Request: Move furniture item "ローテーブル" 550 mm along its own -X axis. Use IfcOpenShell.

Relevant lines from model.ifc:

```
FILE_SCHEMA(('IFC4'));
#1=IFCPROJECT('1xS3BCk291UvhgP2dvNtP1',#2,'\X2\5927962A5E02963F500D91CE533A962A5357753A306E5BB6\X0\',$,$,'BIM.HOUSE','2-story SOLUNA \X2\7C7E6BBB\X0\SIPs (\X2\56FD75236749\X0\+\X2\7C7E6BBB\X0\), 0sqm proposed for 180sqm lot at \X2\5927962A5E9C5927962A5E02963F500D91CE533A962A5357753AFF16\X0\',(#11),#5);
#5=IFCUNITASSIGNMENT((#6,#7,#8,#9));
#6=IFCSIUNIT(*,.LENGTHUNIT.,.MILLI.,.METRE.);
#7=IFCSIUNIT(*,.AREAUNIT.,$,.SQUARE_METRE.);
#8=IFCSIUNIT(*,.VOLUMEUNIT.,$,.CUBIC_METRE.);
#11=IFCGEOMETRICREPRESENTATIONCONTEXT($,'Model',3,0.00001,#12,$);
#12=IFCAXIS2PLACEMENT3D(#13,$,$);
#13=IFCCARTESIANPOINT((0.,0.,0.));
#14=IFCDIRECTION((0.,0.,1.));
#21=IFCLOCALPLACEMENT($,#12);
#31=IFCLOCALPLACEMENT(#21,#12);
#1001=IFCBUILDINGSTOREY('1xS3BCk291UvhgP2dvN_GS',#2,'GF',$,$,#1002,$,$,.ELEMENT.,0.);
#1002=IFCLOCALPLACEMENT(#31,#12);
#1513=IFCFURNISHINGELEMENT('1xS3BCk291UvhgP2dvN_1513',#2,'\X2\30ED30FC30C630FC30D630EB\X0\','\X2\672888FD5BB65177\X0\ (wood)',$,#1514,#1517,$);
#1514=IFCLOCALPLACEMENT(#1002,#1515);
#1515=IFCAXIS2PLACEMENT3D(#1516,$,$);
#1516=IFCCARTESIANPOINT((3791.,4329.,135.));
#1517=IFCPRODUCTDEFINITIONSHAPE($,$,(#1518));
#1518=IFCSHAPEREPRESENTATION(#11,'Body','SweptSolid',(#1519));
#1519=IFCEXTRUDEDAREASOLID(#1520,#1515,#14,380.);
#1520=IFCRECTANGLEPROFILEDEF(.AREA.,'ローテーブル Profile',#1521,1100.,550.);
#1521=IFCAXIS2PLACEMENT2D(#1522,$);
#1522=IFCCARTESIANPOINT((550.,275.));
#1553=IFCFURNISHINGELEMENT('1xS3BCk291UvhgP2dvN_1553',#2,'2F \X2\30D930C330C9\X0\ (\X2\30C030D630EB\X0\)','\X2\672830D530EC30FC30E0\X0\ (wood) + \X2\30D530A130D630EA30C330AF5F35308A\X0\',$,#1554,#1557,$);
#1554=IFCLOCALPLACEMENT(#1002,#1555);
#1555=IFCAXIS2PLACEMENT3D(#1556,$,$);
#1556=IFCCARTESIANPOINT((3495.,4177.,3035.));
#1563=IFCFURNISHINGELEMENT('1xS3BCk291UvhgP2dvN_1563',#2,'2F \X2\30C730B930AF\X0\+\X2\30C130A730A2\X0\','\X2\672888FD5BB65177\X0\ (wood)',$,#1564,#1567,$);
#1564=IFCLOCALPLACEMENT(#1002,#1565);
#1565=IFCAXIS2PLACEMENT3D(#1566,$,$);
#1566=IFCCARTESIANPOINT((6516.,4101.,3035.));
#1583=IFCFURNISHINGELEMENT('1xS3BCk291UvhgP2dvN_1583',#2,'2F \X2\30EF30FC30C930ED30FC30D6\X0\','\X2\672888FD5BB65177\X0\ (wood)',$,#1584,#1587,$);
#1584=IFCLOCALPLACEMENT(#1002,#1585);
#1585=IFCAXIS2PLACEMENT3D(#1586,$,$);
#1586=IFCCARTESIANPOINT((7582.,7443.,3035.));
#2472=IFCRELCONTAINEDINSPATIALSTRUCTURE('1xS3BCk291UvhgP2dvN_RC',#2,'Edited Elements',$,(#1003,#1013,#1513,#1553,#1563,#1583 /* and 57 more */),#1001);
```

```python
import ifcopenshell
import ifcopenshell.api.geometry
import ifcopenshell.util.placement
import ifcopenshell.util.unit

model = ifcopenshell.open("model.ifc")
unit_scale = ifcopenshell.util.unit.calculate_unit_scale(model)

item = model.by_guid("1xS3BCk291UvhgP2dvN_1513")
matrix = ifcopenshell.util.placement.get_local_placement(item.ObjectPlacement)
matrix[:3, 3] -= matrix[:3, 0] * 0.55 / unit_scale
ifcopenshell.api.geometry.edit_object_placement(model, product=item, matrix=matrix, is_si=False)

print(ifcopenshell.util.placement.get_local_placement(item.ObjectPlacement).round(3) + 0.0)

model.write("model_edited.ifc")
```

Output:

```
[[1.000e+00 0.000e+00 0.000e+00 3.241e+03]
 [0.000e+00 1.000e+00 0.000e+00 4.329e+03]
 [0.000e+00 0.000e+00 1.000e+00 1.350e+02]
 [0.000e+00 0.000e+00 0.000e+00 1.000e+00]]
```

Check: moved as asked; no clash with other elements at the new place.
